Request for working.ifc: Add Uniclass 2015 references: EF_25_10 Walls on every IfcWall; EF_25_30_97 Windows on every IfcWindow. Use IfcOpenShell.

First a look at what the model holds.

```python
import ifcopenshell

model = ifcopenshell.open("working.ifc")
print(model.schema)
print("classifications:", [c.Name for c in model.by_type("IfcClassification")])
for ifc_class in ("IfcDoor", "IfcRoof", "IfcStair", "IfcWall", "IfcWindow"):
    print(ifc_class, len(model.by_type(ifc_class)))
```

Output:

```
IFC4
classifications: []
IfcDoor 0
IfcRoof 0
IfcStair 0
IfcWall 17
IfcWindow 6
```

```python
import ifcopenshell
import ifcopenshell.api.classification

model = ifcopenshell.open("working.ifc")

system = ifcopenshell.api.classification.add_classification(model, classification="Uniclass 2015")

codes = {
    "IfcWall": ("EF_25_10", "Walls"),
    "IfcWindow": ("EF_25_30_97", "Windows"),
}
for ifc_class, (code, name) in codes.items():
    products = model.by_type(ifc_class)
    ifcopenshell.api.classification.add_reference(
        model, products=products, classification=system, identification=code, name=name
    )
    print(code, len(products))

model.write("working_v2.ifc")
```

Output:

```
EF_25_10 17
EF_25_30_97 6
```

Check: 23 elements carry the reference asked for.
